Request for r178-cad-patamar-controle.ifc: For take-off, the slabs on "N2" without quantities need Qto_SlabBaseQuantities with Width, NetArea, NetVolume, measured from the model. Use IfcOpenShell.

First a look at what the model holds.

```python
import ifcopenshell
import ifcopenshell.util.element
import ifcopenshell.util.unit

model = ifcopenshell.open("r178-cad-patamar-controle.ifc")
print(model.schema)
for unit_type in ("LENGTHUNIT", "AREAUNIT", "VOLUMEUNIT"):
    print(unit_type, ifcopenshell.util.unit.calculate_unit_scale(model, unit_type))
storey = next(s for s in model.by_type("IfcBuildingStorey") if s.Name == "N2")
slabs = [e for e in ifcopenshell.util.element.get_decomposition(storey) if e.is_a("IfcSlab")]
for e in sorted(slabs, key=lambda e: e.id()):
    print(e.id(), e.is_a(), e.Name, list(ifcopenshell.util.element.get_psets(e, qtos_only=True)), sep=" | ")
```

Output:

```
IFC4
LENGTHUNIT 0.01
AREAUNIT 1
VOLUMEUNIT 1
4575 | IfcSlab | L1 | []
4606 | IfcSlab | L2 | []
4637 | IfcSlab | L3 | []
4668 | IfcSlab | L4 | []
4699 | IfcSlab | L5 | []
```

```python
import ifcopenshell
import ifcopenshell.api.pset
import ifcopenshell.geom
import ifcopenshell.util.element
import ifcopenshell.util.shape
import ifcopenshell.util.unit

model = ifcopenshell.open("r178-cad-patamar-controle.ifc")
unit_scale = ifcopenshell.util.unit.calculate_unit_scale(model)
area_scale = ifcopenshell.util.unit.calculate_unit_scale(model, "AREAUNIT")
volume_scale = ifcopenshell.util.unit.calculate_unit_scale(model, "VOLUMEUNIT")
settings = ifcopenshell.geom.settings()

storey = next(s for s in model.by_type("IfcBuildingStorey") if s.Name == "N2")
slabs = [e for e in ifcopenshell.util.element.get_decomposition(storey) if e.is_a("IfcSlab")]

for e in sorted(slabs, key=lambda e: e.id()):
    if ifcopenshell.util.element.get_psets(e, qtos_only=True, should_inherit=False):
        continue
    # Geometry comes back in metres, in the element's own axes.
    shape = ifcopenshell.geom.create_shape(settings, e)
    values = {
        "Width": ifcopenshell.util.shape.get_z(shape.geometry) / unit_scale,
        "NetArea": ifcopenshell.util.shape.get_footprint_area(shape.geometry) / area_scale,
        "NetVolume": ifcopenshell.util.shape.get_volume(shape.geometry) / volume_scale,
    }
    qto = ifcopenshell.api.pset.add_qto(model, product=e, name="Qto_SlabBaseQuantities")
    ifcopenshell.api.pset.edit_qto(model, qto=qto, properties=values)
    print(e.id(), {k: round(v, 3) for k, v in values.items()})

model.write("r178-cad-patamar-controle_edited.ifc")
```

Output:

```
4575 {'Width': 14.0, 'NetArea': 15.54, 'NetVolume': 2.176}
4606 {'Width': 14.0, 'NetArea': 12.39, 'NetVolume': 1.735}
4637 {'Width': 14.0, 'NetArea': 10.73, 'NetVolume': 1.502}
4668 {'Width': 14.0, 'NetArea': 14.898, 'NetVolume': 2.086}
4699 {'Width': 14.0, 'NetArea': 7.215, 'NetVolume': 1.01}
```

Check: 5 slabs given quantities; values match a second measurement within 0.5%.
